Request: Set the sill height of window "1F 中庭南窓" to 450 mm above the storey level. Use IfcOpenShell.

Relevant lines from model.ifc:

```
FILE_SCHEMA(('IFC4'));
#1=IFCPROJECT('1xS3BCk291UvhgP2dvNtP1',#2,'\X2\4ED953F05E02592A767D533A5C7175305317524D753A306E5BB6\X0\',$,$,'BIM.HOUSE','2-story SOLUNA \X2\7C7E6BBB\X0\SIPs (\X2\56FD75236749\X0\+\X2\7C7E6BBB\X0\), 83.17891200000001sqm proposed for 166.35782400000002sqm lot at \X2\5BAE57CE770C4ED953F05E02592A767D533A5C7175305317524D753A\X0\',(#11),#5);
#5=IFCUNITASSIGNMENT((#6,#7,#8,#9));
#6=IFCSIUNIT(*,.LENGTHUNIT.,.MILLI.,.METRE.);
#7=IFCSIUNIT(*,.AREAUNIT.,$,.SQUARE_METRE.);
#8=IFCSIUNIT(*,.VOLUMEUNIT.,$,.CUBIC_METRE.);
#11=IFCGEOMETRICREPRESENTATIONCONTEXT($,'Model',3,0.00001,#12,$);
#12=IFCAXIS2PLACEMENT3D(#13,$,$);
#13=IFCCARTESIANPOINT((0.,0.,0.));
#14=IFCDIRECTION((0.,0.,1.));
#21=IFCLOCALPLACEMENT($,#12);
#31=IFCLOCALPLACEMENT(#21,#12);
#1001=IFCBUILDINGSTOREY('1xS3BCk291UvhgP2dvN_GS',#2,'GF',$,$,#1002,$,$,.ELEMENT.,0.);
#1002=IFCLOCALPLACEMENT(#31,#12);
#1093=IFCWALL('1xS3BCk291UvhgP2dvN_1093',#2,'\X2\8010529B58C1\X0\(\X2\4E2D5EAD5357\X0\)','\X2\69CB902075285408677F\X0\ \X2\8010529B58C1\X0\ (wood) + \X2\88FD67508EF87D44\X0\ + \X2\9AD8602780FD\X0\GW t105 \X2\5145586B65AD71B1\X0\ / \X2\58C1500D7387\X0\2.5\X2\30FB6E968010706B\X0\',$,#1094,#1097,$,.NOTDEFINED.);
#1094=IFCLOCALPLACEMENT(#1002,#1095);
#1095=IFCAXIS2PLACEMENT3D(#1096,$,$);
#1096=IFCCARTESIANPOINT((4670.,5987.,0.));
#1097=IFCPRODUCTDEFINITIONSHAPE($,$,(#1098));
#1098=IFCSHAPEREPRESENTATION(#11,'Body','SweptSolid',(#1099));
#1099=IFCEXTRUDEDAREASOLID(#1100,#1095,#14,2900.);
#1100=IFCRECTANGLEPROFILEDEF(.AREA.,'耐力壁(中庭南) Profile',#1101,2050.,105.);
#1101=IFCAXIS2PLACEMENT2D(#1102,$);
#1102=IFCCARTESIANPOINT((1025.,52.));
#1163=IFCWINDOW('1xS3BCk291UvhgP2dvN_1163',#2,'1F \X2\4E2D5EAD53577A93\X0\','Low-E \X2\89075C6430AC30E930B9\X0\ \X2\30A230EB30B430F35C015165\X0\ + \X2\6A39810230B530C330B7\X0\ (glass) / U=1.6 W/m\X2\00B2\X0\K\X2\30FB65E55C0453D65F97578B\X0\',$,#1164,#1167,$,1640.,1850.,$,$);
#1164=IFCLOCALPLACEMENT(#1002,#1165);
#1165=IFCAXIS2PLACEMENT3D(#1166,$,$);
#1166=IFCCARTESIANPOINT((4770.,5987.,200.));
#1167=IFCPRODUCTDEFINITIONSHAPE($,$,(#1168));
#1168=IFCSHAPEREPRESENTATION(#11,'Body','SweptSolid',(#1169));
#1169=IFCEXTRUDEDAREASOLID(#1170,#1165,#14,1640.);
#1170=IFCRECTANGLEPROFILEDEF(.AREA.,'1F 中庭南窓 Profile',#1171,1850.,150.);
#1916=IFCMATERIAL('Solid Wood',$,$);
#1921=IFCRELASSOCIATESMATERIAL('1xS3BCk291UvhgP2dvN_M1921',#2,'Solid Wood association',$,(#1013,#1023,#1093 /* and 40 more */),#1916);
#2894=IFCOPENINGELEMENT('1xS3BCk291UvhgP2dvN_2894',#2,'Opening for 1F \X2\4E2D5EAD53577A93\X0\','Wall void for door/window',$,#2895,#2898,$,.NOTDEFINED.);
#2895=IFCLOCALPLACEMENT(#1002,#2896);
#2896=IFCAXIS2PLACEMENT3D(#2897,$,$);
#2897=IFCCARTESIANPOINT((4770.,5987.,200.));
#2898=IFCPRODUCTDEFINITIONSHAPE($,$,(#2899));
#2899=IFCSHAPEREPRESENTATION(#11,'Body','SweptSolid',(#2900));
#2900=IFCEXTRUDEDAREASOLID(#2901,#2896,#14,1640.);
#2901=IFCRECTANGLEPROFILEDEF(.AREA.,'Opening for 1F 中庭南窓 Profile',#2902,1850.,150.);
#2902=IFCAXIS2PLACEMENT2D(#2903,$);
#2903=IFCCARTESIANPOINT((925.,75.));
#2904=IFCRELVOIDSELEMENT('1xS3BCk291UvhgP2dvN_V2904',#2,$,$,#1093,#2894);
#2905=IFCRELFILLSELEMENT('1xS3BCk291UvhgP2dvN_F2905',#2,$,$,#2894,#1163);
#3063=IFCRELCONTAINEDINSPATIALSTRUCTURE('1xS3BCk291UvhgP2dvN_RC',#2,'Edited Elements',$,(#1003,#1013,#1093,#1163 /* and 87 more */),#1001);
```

```python
import numpy as np
import ifcopenshell
import ifcopenshell.api.geometry
import ifcopenshell.geom
import ifcopenshell.util.element
import ifcopenshell.util.placement
import ifcopenshell.util.shape
import ifcopenshell.util.unit

model = ifcopenshell.open("model.ifc")
unit_scale = ifcopenshell.util.unit.calculate_unit_scale(model)

window = model.by_guid("1xS3BCk291UvhgP2dvN_1163")
opening = window.FillsVoids[0].RelatingOpeningElement
storey = ifcopenshell.util.element.get_container(window, ifc_class="IfcBuildingStorey")
level = ifcopenshell.util.placement.get_local_placement(storey.ObjectPlacement)[2, 3]

# The opening's origin need not be at the sill, so measure its lowest point.
shape = ifcopenshell.geom.create_shape(ifcopenshell.geom.settings(), opening)
bottom = ifcopenshell.util.shape.get_shape_bottom_elevation(shape, shape.geometry) / unit_scale
dz = level + 450.0 - bottom

shift = np.array([0.0, 0.0, dz])
# The window is not placed relative to its opening, so move both.
for product in (opening, window):
    matrix = ifcopenshell.util.placement.get_local_placement(product.ObjectPlacement)
    matrix[:3, 3] += shift
    ifcopenshell.api.geometry.edit_object_placement(model, product=product, matrix=matrix, is_si=False)

print(f"moved by {dz * unit_scale:+.3f} m")

model.write("model_updated.ifc")
```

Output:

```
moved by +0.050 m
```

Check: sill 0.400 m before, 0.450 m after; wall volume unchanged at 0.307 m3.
